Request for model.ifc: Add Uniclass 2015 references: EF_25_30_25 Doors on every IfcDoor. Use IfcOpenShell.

First a look at what the model holds.

```python
import ifcopenshell

model = ifcopenshell.open("model.ifc")
print(model.schema)
print("classifications:", [c.Name for c in model.by_type("IfcClassification")])
for ifc_class in ("IfcDoor", "IfcRoof", "IfcStair", "IfcWall", "IfcWindow"):
    print(ifc_class, len(model.by_type(ifc_class)))
```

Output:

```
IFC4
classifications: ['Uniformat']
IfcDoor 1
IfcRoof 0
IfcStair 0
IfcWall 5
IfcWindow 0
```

```python
import ifcopenshell
import ifcopenshell.api.classification

model = ifcopenshell.open("model.ifc")

system = ifcopenshell.api.classification.add_classification(model, classification="Uniclass 2015")

codes = {
    "IfcDoor": ("EF_25_30_25", "Doors"),
}
for ifc_class, (code, name) in codes.items():
    products = model.by_type(ifc_class)
    ifcopenshell.api.classification.add_reference(
        model, products=products, classification=system, identification=code, name=name
    )
    print(code, len(products))

model.write("model_updated.ifc")
```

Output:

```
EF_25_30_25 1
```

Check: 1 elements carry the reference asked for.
